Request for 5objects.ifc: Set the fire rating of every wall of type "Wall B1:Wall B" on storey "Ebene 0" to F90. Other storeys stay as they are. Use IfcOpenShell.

First a look at what the model holds.

```python
import ifcopenshell
import ifcopenshell.util.element

model = ifcopenshell.open("5objects.ifc")
print(model.schema)
storey = next(s for s in model.by_type("IfcBuildingStorey") if s.Name == "Ebene 0")
walls = [e for e in ifcopenshell.util.element.get_decomposition(storey) if e.is_a("IfcWall")]
seen = {}
for e in walls:
    element_type = ifcopenshell.util.element.get_type(e)
    key = (element_type.Name if element_type != e and element_type else None, ifcopenshell.util.element.get_pset(e, "Pset_WallCommon", "FireRating"))
    seen[key] = seen.get(key, 0) + 1
for (name, value), count in sorted(seen.items(), key=str):
    print(count, "x", name, "|", value)
```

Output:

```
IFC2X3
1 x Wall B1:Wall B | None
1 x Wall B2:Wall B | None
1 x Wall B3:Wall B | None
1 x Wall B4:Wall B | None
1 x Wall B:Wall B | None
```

```python
import ifcopenshell
import ifcopenshell.api.pset
import ifcopenshell.util.element

model = ifcopenshell.open("5objects.ifc")

storey = next(s for s in model.by_type("IfcBuildingStorey") if s.Name == "Ebene 0")
walls = [e for e in ifcopenshell.util.element.get_decomposition(storey) if e.is_a("IfcWall")]

count = 0
for e in walls:
    element_type = ifcopenshell.util.element.get_type(e)
    if element_type in (None, e) or element_type.Name != "Wall B1:Wall B":
        continue
    # add_pset returns the element's existing set when there is one.
    pset = ifcopenshell.api.pset.add_pset(model, product=e, name="Pset_WallCommon")
    ifcopenshell.api.pset.edit_pset(model, pset=pset, properties={"FireRating": "F90"})
    count += 1

print(count, "walls updated")

model.write("5objects_rev.ifc")
```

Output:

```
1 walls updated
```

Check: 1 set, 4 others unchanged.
